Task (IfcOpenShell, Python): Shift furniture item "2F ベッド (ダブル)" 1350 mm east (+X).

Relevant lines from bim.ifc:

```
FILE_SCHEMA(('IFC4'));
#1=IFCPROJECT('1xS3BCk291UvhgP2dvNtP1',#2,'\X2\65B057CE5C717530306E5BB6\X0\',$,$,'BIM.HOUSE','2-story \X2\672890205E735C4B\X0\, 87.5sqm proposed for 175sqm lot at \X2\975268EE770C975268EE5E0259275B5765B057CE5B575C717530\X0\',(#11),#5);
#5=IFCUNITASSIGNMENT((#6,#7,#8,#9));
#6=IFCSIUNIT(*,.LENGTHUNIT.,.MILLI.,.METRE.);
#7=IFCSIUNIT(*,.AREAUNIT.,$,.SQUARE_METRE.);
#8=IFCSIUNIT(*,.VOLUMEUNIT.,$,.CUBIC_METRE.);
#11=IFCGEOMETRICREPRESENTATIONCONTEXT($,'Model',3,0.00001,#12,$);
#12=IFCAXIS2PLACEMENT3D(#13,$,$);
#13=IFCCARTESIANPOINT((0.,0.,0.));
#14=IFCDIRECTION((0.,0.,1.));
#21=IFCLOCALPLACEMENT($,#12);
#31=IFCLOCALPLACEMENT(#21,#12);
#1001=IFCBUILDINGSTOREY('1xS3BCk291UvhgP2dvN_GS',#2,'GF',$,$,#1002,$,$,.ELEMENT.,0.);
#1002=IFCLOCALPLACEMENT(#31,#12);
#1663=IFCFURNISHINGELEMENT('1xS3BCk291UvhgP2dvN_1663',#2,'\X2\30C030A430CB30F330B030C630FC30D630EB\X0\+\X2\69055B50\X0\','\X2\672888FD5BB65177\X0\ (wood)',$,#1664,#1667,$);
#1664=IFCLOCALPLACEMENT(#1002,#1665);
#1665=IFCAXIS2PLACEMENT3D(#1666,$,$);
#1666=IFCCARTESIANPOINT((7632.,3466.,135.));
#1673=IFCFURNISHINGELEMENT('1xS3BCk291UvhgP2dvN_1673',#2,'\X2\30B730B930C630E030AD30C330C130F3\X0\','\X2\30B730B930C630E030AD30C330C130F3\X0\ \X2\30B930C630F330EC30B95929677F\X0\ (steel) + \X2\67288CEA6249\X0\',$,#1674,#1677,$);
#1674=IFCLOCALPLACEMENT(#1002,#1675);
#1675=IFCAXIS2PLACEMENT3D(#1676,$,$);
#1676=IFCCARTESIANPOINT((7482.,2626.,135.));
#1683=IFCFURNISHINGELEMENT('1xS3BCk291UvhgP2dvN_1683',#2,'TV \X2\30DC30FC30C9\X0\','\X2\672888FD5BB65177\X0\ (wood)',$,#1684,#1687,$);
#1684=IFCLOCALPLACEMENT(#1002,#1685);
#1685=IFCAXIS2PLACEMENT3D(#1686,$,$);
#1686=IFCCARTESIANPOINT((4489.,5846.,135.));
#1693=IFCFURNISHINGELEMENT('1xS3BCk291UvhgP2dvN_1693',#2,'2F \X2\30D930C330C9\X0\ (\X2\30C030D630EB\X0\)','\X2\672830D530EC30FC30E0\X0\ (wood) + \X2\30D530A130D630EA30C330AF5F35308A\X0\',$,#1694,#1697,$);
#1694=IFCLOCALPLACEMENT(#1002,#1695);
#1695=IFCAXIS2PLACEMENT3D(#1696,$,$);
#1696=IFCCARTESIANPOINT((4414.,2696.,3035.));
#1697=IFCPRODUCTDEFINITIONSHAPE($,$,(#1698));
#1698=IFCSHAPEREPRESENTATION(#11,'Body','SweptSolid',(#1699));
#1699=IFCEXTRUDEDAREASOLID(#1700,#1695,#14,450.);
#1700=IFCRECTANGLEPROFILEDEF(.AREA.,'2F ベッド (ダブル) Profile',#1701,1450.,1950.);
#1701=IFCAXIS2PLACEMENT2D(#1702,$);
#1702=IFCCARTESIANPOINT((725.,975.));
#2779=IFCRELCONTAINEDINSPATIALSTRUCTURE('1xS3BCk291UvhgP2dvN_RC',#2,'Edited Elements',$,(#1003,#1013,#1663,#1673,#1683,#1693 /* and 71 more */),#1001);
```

```python
import ifcopenshell
import ifcopenshell.api.geometry
import ifcopenshell.util.placement
import ifcopenshell.util.unit

model = ifcopenshell.open("bim.ifc")
unit_scale = ifcopenshell.util.unit.calculate_unit_scale(model)

item = model.by_id(1693)
matrix = ifcopenshell.util.placement.get_local_placement(item.ObjectPlacement)
matrix[0, 3] += 1.35 / unit_scale
ifcopenshell.api.geometry.edit_object_placement(model, product=item, matrix=matrix, is_si=False)

print(ifcopenshell.util.placement.get_local_placement(item.ObjectPlacement).round(3) + 0.0)

model.write("bim_edited.ifc")
```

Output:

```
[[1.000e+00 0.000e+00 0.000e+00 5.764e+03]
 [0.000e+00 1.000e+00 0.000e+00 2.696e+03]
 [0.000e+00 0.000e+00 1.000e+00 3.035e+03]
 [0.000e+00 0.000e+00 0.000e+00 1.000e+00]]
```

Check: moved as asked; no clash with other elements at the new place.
